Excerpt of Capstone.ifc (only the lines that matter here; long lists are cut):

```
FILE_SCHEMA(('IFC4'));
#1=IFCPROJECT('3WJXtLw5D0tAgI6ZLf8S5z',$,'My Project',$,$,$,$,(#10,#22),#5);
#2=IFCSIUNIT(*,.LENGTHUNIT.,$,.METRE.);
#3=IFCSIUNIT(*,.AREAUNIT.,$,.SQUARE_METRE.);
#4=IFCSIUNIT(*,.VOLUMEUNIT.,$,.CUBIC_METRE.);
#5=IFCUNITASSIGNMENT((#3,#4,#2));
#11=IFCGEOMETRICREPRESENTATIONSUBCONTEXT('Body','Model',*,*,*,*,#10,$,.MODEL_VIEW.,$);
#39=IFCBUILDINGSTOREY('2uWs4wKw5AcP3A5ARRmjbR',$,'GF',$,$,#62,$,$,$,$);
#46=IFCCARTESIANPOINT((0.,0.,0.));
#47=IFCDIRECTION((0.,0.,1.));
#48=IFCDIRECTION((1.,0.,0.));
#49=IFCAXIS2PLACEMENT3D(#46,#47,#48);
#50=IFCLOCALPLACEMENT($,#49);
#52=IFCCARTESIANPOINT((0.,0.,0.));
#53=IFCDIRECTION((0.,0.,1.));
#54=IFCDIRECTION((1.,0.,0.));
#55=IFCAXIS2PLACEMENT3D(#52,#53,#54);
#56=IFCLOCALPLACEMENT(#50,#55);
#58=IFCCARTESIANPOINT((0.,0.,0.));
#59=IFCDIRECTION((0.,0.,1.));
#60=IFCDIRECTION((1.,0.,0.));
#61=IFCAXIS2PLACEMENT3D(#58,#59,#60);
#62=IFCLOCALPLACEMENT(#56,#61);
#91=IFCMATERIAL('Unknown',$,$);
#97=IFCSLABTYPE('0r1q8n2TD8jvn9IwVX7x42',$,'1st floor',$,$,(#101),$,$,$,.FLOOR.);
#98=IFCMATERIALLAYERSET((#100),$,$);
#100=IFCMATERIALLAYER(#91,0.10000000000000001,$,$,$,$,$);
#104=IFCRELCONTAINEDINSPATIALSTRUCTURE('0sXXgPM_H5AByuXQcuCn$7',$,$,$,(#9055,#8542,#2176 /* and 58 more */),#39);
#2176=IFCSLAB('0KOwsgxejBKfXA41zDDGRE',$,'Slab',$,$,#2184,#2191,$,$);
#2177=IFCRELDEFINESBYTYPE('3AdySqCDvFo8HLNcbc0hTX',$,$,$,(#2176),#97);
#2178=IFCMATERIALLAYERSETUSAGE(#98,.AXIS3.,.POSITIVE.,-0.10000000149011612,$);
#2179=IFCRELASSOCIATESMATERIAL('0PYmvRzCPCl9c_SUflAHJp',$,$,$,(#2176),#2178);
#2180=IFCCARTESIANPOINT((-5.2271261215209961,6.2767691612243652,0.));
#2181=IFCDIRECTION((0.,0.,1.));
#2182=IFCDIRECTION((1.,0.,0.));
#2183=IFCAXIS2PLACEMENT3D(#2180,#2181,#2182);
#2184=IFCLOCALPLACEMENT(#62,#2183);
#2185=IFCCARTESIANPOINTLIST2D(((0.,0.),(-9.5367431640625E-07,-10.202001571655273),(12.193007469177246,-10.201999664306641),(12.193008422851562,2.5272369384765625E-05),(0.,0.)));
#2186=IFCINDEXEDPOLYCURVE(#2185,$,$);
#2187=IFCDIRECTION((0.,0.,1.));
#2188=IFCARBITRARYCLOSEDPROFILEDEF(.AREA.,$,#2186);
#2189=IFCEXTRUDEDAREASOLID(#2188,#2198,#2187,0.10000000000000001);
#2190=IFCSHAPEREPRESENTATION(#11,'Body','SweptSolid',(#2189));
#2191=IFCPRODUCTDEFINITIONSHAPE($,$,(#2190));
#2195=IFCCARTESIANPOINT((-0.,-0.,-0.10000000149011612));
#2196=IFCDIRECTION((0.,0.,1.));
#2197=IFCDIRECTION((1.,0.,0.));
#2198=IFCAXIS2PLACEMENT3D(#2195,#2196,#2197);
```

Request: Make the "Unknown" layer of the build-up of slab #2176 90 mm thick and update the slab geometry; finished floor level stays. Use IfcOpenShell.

```python
import ifcopenshell
import ifcopenshell.util.element
import ifcopenshell.util.representation

model = ifcopenshell.open("Capstone.ifc")

layer_set = model.by_id(98)
layer = next(l for l in layer_set.MaterialLayers if l.Material and l.Material.Name == "Unknown")
change = 0.09 - layer.LayerThickness
layer.LayerThickness += change

# Geometry does not follow the layer set by itself.
slabs = [e for e in ifcopenshell.util.element.get_elements_by_material(model, layer_set) if e.is_a("IfcSlab")]
for slab in sorted(slabs, key=lambda e: e.id()):
    body = ifcopenshell.util.representation.get_representation(slab, "Model", "Body")
    solid = body.Items[0]
    old_depth = solid.Depth
    solid.Depth += change
    # Extruded upwards: lower the start of the extrusion so the top stays.
    x, y, z = solid.Position.Location.Coordinates
    solid.Position.Location = model.createIfcCartesianPoint((x, y, z - change))
    print(slab.id(), f"{old_depth:g} -> {solid.Depth:g}")

# The layers are counted up from the underside, which has moved.
for usage in {ifcopenshell.util.element.get_material(slab) for slab in slabs}:
    usage.OffsetFromReferenceLine -= change

model.write("Capstone-out.ifc")
```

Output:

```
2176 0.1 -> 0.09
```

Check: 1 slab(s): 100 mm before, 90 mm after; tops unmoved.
